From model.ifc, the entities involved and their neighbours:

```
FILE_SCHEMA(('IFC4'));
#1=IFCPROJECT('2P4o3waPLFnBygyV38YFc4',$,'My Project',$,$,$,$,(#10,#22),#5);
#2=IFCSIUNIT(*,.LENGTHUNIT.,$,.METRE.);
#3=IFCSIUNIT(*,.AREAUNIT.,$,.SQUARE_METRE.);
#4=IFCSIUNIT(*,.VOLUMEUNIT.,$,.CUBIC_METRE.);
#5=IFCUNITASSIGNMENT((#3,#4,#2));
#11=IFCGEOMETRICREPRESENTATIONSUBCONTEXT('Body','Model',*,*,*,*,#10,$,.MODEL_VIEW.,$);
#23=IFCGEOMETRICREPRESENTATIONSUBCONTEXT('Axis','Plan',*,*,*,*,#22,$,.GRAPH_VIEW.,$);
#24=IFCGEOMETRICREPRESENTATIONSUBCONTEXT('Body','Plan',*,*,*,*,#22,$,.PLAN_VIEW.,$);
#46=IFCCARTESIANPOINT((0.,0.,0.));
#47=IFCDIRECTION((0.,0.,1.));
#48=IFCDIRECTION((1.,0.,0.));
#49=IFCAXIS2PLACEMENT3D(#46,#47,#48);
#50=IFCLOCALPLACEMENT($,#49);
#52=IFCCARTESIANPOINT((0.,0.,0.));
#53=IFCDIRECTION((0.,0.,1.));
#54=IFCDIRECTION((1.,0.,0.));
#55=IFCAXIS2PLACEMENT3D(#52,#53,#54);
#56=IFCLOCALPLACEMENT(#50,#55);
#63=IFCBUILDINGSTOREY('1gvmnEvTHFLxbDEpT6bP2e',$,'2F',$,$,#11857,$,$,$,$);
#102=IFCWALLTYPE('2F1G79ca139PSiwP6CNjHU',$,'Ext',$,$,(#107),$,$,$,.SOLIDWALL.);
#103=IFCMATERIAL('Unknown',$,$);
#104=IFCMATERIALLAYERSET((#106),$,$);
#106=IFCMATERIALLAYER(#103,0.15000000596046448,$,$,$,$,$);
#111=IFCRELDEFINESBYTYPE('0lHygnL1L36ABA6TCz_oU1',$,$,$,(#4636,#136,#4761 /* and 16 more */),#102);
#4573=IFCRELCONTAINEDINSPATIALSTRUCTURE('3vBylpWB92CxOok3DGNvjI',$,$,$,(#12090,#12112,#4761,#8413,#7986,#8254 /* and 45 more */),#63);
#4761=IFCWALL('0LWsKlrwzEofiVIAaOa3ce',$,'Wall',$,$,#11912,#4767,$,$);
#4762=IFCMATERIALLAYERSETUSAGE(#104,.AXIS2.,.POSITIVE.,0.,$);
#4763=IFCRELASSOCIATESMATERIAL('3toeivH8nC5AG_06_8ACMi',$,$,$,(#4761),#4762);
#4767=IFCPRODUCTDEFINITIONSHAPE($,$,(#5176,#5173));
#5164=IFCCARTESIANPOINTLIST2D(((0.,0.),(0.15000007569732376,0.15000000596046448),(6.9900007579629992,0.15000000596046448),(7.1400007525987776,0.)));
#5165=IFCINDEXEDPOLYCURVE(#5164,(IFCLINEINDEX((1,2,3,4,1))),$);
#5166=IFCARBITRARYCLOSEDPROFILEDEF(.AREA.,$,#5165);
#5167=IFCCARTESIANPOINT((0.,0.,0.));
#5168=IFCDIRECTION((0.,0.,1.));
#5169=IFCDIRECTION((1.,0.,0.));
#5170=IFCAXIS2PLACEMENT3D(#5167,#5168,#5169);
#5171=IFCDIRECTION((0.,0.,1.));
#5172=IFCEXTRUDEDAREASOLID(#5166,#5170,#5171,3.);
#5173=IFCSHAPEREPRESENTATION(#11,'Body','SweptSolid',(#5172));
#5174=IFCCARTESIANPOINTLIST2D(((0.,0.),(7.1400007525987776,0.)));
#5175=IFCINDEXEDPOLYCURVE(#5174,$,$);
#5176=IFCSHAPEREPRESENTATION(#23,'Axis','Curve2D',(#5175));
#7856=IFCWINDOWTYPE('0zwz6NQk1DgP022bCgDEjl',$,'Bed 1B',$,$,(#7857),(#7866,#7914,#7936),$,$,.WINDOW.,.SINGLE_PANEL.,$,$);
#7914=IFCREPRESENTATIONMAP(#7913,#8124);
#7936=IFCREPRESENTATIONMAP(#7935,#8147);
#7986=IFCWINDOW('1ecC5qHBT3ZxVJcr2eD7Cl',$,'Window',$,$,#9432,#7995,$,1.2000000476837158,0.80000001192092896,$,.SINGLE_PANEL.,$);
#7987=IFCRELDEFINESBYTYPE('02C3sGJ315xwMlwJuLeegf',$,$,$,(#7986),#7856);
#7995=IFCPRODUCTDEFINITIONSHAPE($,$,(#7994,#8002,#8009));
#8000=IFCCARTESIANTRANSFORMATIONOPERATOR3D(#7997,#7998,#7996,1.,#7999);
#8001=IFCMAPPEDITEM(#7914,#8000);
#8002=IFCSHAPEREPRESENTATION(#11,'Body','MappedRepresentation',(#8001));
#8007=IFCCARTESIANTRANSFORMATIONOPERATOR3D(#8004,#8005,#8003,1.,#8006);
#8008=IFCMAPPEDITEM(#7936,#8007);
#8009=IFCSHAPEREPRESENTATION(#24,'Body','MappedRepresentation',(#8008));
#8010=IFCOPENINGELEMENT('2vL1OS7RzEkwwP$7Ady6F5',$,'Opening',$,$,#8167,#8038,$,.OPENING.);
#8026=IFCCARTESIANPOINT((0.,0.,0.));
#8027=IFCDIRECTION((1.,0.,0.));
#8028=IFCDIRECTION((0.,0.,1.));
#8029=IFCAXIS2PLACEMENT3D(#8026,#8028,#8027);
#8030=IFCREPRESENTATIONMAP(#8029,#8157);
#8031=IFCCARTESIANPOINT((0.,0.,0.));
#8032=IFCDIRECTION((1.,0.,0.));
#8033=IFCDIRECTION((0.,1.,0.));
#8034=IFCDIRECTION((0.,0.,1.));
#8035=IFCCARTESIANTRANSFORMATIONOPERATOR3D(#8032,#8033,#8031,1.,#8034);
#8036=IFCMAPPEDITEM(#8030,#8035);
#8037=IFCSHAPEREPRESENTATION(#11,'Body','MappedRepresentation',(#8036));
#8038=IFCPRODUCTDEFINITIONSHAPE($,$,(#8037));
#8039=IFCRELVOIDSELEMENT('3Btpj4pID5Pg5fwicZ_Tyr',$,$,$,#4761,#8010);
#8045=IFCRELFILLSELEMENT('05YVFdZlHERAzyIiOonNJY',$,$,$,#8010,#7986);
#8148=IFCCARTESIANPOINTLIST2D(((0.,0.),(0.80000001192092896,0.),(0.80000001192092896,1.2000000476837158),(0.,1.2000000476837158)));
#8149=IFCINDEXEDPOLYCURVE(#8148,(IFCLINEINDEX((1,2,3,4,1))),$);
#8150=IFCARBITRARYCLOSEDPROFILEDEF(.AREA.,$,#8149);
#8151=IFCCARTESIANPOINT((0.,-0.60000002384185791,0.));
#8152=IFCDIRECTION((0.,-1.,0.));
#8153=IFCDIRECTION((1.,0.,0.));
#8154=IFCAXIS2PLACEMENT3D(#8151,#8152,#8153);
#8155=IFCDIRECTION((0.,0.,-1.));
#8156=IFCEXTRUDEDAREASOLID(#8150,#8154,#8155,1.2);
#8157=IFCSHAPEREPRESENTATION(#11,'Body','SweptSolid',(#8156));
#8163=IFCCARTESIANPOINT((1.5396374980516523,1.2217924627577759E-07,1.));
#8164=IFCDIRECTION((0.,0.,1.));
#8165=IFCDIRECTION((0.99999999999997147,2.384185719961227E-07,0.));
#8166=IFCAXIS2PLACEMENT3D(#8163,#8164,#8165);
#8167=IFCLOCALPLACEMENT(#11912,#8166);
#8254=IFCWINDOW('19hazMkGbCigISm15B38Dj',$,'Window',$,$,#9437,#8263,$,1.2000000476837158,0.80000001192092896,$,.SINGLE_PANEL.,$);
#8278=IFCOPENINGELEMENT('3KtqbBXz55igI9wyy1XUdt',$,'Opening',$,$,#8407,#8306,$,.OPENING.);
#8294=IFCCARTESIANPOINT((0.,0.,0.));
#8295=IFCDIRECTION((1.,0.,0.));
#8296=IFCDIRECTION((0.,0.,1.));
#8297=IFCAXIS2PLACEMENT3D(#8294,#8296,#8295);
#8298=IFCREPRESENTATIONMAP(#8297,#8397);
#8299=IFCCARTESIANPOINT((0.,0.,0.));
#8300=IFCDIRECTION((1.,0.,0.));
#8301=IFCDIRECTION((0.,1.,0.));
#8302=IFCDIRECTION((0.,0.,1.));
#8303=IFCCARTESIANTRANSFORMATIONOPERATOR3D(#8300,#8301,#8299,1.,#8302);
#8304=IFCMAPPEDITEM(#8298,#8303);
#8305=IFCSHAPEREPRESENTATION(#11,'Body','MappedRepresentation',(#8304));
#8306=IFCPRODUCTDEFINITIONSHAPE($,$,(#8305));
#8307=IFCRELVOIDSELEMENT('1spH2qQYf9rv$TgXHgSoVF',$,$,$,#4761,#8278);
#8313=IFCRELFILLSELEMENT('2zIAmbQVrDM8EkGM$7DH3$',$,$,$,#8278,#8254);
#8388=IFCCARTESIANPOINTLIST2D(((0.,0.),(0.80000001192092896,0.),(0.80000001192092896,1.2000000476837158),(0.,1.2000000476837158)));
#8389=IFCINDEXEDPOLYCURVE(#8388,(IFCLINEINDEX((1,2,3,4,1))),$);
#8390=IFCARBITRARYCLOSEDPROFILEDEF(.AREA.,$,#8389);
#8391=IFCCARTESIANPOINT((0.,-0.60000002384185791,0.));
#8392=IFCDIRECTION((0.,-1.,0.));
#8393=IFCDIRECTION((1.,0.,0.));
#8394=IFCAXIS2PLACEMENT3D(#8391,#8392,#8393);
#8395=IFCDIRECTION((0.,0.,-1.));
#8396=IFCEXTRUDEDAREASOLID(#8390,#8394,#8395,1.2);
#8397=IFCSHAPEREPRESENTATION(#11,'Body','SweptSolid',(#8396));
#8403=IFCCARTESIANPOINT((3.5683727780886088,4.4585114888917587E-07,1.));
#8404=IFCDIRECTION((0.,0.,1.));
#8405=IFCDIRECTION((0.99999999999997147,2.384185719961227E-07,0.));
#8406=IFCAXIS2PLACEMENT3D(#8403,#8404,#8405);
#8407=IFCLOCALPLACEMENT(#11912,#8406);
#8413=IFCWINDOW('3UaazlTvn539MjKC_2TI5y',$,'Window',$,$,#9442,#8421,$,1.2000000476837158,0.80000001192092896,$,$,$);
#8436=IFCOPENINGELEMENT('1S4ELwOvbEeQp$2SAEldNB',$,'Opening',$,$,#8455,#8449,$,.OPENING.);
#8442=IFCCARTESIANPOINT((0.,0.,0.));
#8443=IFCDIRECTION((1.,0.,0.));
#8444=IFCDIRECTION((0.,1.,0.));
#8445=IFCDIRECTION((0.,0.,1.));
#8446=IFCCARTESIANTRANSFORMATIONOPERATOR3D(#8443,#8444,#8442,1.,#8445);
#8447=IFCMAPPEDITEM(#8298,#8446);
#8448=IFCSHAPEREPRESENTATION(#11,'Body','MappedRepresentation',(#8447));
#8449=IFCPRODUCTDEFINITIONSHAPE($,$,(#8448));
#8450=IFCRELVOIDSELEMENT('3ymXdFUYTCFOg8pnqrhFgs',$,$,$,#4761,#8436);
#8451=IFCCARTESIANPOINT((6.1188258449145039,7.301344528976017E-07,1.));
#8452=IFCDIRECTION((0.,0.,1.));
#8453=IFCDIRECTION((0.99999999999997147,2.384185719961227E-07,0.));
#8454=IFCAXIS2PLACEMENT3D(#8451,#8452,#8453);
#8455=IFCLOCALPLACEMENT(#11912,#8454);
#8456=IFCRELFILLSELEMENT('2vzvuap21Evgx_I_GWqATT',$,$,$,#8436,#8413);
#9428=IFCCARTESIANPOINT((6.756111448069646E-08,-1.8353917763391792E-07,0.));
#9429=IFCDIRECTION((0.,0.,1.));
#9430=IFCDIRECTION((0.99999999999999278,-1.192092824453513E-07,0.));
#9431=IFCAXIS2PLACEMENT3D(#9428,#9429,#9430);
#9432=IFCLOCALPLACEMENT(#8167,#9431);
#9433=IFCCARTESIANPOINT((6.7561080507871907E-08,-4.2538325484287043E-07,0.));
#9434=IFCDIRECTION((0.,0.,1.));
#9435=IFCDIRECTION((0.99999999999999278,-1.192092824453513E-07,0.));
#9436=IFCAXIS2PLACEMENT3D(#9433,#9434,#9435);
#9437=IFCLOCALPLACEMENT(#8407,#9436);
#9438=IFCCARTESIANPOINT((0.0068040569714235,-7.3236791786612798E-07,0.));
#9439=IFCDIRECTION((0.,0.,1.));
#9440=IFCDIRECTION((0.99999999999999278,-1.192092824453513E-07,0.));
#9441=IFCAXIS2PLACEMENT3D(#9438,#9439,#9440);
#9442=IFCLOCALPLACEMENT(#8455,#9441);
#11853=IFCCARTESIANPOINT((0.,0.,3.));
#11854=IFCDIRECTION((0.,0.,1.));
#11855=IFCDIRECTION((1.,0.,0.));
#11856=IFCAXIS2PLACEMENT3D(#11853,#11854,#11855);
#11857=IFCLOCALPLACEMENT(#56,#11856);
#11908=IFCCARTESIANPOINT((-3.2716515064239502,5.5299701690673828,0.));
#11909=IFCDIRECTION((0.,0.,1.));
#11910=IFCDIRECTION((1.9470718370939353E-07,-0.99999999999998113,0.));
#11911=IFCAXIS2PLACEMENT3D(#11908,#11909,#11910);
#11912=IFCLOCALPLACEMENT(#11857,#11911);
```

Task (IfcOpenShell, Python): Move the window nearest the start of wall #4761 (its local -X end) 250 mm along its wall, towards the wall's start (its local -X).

```python
import ifcopenshell
import ifcopenshell.api.geometry
import ifcopenshell.util.placement
import ifcopenshell.util.unit

model = ifcopenshell.open("model.ifc")
unit_scale = ifcopenshell.util.unit.calculate_unit_scale(model)

window = model.by_guid("1ecC5qHBT3ZxVJcr2eD7Cl")
opening = window.FillsVoids[0].RelatingOpeningElement
wall = opening.VoidsElements[0].RelatingBuildingElement

wall_matrix = ifcopenshell.util.placement.get_local_placement(wall.ObjectPlacement)
shift = wall_matrix[:3, 0] * -0.25 / unit_scale
before = ifcopenshell.util.placement.get_local_placement(window.ObjectPlacement)[:3, 3].copy()

# The window is placed relative to its opening, so it follows when the opening moves.
matrix = ifcopenshell.util.placement.get_local_placement(opening.ObjectPlacement)
matrix[:3, 3] += shift
ifcopenshell.api.geometry.edit_object_placement(
    model, product=opening, matrix=matrix, is_si=False, should_transform_children=True
)

after = ifcopenshell.util.placement.get_local_placement(window.ObjectPlacement)[:3, 3]
print("window moved by", (after - before).round(3) + 0.0)

model.write("model_updated.ifc")
```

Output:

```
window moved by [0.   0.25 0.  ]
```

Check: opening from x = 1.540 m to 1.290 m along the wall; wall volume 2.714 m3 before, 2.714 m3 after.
